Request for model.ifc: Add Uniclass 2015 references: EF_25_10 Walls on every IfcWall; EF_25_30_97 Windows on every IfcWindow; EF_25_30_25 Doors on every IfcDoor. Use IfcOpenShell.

First a look at what the model holds.

```python
import ifcopenshell

model = ifcopenshell.open("model.ifc")
print(model.schema)
print("classifications:", [c.Name for c in model.by_type("IfcClassification")])
for ifc_class in ("IfcDoor", "IfcRoof", "IfcStair", "IfcWall", "IfcWindow"):
    print(ifc_class, len(model.by_type(ifc_class)))
```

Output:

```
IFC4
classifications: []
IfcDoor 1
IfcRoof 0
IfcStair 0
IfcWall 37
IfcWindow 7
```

```python
import ifcopenshell
import ifcopenshell.api.classification

model = ifcopenshell.open("model.ifc")

system = ifcopenshell.api.classification.add_classification(model, classification="Uniclass 2015")

codes = {
    "IfcWall": ("EF_25_10", "Walls"),
    "IfcWindow": ("EF_25_30_97", "Windows"),
    "IfcDoor": ("EF_25_30_25", "Doors"),
}
for ifc_class, (code, name) in codes.items():
    products = model.by_type(ifc_class)
    ifcopenshell.api.classification.add_reference(
        model, products=products, classification=system, identification=code, name=name
    )
    print(code, len(products))

model.write("model_edited.ifc")
```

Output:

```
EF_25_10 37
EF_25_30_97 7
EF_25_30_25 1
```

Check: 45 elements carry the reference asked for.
